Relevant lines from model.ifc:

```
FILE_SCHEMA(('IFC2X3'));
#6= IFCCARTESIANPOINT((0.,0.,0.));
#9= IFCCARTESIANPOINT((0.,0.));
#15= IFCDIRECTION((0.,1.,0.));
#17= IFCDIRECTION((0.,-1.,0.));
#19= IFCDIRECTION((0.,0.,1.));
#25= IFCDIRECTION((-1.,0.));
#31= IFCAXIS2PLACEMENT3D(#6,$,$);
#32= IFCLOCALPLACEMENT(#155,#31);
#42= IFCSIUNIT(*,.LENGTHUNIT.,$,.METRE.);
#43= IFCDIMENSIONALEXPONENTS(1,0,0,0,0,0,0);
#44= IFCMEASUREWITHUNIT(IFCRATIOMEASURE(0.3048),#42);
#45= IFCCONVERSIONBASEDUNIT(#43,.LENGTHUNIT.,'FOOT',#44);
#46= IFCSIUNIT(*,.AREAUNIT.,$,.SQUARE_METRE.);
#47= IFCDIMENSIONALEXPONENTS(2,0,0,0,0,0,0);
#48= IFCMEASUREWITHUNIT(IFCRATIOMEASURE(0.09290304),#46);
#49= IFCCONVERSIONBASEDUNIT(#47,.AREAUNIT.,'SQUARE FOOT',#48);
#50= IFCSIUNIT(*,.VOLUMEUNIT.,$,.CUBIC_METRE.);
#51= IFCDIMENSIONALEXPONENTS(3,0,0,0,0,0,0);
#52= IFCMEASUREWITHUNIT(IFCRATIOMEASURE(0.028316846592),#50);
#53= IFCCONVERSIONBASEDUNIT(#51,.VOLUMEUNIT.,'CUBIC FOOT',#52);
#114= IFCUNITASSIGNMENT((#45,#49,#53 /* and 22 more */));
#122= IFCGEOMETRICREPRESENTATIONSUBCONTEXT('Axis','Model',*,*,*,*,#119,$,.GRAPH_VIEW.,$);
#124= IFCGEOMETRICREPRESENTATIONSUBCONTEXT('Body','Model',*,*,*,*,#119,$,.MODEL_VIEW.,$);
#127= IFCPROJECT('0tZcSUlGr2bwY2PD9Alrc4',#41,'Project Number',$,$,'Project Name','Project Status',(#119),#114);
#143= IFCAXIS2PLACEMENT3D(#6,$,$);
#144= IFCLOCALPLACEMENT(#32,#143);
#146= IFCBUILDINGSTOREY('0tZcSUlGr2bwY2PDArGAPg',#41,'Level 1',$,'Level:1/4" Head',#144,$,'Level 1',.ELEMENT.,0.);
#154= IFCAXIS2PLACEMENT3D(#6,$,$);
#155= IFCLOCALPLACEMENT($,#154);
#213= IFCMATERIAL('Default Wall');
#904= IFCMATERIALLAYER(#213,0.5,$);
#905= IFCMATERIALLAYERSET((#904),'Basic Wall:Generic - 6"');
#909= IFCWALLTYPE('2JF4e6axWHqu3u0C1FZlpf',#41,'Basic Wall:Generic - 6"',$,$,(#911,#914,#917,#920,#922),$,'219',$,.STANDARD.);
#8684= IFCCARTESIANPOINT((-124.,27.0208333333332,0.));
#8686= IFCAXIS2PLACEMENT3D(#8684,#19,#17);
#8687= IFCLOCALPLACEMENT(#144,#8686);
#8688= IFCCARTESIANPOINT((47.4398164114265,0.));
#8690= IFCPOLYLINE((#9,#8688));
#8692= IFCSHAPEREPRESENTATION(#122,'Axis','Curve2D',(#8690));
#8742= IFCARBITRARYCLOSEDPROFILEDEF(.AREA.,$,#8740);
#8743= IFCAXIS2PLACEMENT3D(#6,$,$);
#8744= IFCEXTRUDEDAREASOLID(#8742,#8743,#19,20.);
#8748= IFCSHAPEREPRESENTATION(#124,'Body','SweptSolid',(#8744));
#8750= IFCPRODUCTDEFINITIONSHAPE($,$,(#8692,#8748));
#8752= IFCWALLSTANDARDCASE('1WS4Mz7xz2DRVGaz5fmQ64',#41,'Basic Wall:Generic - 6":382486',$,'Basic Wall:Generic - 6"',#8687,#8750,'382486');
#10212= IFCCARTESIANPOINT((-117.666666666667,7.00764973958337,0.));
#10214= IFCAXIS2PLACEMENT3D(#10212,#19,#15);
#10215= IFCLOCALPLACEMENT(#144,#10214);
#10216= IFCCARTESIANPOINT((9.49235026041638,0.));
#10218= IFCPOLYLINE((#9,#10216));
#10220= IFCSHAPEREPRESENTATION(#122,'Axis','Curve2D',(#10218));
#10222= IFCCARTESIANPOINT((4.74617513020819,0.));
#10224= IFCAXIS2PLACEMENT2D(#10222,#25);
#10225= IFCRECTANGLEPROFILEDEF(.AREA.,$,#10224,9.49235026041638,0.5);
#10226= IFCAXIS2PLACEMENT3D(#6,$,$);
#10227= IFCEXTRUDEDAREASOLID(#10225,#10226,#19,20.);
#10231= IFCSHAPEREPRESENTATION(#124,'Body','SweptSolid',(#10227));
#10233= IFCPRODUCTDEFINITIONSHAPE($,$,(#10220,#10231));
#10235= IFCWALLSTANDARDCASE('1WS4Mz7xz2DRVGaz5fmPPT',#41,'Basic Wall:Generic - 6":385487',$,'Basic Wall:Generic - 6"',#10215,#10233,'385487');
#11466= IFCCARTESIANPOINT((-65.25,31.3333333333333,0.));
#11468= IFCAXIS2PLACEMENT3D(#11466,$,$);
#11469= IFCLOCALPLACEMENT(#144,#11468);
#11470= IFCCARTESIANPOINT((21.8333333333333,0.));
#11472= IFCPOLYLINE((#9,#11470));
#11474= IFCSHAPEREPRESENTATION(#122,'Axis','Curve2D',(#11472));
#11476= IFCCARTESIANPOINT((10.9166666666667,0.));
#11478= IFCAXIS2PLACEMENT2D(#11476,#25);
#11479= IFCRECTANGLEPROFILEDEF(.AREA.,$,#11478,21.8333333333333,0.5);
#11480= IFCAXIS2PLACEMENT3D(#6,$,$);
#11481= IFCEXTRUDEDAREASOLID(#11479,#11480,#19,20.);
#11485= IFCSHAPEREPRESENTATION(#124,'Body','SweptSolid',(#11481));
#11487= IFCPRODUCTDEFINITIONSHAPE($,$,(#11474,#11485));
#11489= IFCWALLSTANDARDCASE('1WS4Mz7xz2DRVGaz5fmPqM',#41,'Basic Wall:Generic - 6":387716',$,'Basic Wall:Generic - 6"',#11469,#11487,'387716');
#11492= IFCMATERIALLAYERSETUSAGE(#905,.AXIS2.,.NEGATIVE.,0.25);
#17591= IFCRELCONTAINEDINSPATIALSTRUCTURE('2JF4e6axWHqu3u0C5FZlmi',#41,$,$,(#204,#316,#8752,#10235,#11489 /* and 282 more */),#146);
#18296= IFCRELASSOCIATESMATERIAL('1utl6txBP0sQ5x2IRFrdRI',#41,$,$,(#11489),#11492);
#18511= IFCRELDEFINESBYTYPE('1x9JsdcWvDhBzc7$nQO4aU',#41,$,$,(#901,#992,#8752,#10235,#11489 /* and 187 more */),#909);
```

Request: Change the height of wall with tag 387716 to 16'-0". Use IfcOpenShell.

```python
import ifcopenshell
import ifcopenshell.geom
import ifcopenshell.util.representation
import ifcopenshell.util.shape
import ifcopenshell.util.unit

model = ifcopenshell.open("model.ifc")
unit_scale = ifcopenshell.util.unit.calculate_unit_scale(model)
settings = ifcopenshell.geom.settings()


def volume(element):
    """Net volume in cubic metres, openings subtracted."""
    shape = ifcopenshell.geom.create_shape(settings, element)
    return ifcopenshell.util.shape.get_volume(shape.geometry)


wall = model.by_id(11489)
before = volume(wall)

body = ifcopenshell.util.representation.get_representation(wall, "Model", "Body")
solid = body.Items[0]
old_height = solid.Depth
solid.Depth = 192 * 0.0254 / unit_scale
after = volume(wall)

print(f"height {old_height:g} -> {solid.Depth:g}, volume {before:.3f} -> {after:.3f} m3")

model.write("model_edited.ifc")
```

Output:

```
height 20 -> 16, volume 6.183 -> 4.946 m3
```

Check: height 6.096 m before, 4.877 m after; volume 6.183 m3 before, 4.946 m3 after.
